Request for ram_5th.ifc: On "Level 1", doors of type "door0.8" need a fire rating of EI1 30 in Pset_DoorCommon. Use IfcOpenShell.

First a look at what the model holds.

```python
import ifcopenshell
import ifcopenshell.util.element

model = ifcopenshell.open("ram_5th.ifc")
print(model.schema)
storey = next(s for s in model.by_type("IfcBuildingStorey") if s.Name == "Level 1")
doors = [e for e in ifcopenshell.util.element.get_decomposition(storey) if e.is_a("IfcDoor")]
seen = {}
for e in doors:
    element_type = ifcopenshell.util.element.get_type(e)
    key = (element_type.Name if element_type != e and element_type else None, ifcopenshell.util.element.get_pset(e, "Pset_DoorCommon", "FireRating"))
    seen[key] = seen.get(key, 0) + 1
for (name, value), count in sorted(seen.items(), key=str):
    print(count, "x", name, "|", value)
```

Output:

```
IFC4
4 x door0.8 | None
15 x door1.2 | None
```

```python
import ifcopenshell
import ifcopenshell.api.pset
import ifcopenshell.util.element

model = ifcopenshell.open("ram_5th.ifc")

storey = next(s for s in model.by_type("IfcBuildingStorey") if s.Name == "Level 1")
doors = [e for e in ifcopenshell.util.element.get_decomposition(storey) if e.is_a("IfcDoor")]

count = 0
for e in doors:
    element_type = ifcopenshell.util.element.get_type(e)
    if element_type in (None, e) or element_type.Name != "door0.8":
        continue
    # add_pset returns the element's existing set when there is one.
    pset = ifcopenshell.api.pset.add_pset(model, product=e, name="Pset_DoorCommon")
    ifcopenshell.api.pset.edit_pset(model, pset=pset, properties={"FireRating": "EI1 30"})
    count += 1

print(count, "doors updated")

model.write("ram_5th-out.ifc")
```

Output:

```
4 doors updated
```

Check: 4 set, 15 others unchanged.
